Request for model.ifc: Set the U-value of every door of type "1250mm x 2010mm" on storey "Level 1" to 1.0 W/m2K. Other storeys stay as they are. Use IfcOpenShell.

First a look at what the model holds.

```python
import ifcopenshell
import ifcopenshell.util.element

model = ifcopenshell.open("model.ifc")
print(model.schema)
storey = next(s for s in model.by_type("IfcBuildingStorey") if s.Name == "Level 1")
doors = [e for e in ifcopenshell.util.element.get_decomposition(storey) if e.is_a("IfcDoor")]
seen = {}
for e in doors:
    element_type = ifcopenshell.util.element.get_type(e)
    key = (element_type.Name if element_type != e and element_type else None, ifcopenshell.util.element.get_pset(e, "Pset_DoorCommon", "ThermalTransmittance"))
    seen[key] = seen.get(key, 0) + 1
for (name, value), count in sorted(seen.items(), key=str):
    print(count, "x", name, "|", value)
```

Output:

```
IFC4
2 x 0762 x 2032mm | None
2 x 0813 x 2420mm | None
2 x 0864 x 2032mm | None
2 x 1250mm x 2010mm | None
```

```python
import ifcopenshell
import ifcopenshell.api.pset
import ifcopenshell.util.element

model = ifcopenshell.open("model.ifc")

storey = next(s for s in model.by_type("IfcBuildingStorey") if s.Name == "Level 1")
doors = [e for e in ifcopenshell.util.element.get_decomposition(storey) if e.is_a("IfcDoor")]

count = 0
for e in doors:
    element_type = ifcopenshell.util.element.get_type(e)
    if element_type in (None, e) or element_type.Name != "1250mm x 2010mm":
        continue
    # add_pset returns the element's existing set when there is one.
    pset = ifcopenshell.api.pset.add_pset(model, product=e, name="Pset_DoorCommon")
    ifcopenshell.api.pset.edit_pset(model, pset=pset, properties={"ThermalTransmittance": 1.0})
    count += 1

print(count, "doors updated")

model.write("model-out.ifc")
```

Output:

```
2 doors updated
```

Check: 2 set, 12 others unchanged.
